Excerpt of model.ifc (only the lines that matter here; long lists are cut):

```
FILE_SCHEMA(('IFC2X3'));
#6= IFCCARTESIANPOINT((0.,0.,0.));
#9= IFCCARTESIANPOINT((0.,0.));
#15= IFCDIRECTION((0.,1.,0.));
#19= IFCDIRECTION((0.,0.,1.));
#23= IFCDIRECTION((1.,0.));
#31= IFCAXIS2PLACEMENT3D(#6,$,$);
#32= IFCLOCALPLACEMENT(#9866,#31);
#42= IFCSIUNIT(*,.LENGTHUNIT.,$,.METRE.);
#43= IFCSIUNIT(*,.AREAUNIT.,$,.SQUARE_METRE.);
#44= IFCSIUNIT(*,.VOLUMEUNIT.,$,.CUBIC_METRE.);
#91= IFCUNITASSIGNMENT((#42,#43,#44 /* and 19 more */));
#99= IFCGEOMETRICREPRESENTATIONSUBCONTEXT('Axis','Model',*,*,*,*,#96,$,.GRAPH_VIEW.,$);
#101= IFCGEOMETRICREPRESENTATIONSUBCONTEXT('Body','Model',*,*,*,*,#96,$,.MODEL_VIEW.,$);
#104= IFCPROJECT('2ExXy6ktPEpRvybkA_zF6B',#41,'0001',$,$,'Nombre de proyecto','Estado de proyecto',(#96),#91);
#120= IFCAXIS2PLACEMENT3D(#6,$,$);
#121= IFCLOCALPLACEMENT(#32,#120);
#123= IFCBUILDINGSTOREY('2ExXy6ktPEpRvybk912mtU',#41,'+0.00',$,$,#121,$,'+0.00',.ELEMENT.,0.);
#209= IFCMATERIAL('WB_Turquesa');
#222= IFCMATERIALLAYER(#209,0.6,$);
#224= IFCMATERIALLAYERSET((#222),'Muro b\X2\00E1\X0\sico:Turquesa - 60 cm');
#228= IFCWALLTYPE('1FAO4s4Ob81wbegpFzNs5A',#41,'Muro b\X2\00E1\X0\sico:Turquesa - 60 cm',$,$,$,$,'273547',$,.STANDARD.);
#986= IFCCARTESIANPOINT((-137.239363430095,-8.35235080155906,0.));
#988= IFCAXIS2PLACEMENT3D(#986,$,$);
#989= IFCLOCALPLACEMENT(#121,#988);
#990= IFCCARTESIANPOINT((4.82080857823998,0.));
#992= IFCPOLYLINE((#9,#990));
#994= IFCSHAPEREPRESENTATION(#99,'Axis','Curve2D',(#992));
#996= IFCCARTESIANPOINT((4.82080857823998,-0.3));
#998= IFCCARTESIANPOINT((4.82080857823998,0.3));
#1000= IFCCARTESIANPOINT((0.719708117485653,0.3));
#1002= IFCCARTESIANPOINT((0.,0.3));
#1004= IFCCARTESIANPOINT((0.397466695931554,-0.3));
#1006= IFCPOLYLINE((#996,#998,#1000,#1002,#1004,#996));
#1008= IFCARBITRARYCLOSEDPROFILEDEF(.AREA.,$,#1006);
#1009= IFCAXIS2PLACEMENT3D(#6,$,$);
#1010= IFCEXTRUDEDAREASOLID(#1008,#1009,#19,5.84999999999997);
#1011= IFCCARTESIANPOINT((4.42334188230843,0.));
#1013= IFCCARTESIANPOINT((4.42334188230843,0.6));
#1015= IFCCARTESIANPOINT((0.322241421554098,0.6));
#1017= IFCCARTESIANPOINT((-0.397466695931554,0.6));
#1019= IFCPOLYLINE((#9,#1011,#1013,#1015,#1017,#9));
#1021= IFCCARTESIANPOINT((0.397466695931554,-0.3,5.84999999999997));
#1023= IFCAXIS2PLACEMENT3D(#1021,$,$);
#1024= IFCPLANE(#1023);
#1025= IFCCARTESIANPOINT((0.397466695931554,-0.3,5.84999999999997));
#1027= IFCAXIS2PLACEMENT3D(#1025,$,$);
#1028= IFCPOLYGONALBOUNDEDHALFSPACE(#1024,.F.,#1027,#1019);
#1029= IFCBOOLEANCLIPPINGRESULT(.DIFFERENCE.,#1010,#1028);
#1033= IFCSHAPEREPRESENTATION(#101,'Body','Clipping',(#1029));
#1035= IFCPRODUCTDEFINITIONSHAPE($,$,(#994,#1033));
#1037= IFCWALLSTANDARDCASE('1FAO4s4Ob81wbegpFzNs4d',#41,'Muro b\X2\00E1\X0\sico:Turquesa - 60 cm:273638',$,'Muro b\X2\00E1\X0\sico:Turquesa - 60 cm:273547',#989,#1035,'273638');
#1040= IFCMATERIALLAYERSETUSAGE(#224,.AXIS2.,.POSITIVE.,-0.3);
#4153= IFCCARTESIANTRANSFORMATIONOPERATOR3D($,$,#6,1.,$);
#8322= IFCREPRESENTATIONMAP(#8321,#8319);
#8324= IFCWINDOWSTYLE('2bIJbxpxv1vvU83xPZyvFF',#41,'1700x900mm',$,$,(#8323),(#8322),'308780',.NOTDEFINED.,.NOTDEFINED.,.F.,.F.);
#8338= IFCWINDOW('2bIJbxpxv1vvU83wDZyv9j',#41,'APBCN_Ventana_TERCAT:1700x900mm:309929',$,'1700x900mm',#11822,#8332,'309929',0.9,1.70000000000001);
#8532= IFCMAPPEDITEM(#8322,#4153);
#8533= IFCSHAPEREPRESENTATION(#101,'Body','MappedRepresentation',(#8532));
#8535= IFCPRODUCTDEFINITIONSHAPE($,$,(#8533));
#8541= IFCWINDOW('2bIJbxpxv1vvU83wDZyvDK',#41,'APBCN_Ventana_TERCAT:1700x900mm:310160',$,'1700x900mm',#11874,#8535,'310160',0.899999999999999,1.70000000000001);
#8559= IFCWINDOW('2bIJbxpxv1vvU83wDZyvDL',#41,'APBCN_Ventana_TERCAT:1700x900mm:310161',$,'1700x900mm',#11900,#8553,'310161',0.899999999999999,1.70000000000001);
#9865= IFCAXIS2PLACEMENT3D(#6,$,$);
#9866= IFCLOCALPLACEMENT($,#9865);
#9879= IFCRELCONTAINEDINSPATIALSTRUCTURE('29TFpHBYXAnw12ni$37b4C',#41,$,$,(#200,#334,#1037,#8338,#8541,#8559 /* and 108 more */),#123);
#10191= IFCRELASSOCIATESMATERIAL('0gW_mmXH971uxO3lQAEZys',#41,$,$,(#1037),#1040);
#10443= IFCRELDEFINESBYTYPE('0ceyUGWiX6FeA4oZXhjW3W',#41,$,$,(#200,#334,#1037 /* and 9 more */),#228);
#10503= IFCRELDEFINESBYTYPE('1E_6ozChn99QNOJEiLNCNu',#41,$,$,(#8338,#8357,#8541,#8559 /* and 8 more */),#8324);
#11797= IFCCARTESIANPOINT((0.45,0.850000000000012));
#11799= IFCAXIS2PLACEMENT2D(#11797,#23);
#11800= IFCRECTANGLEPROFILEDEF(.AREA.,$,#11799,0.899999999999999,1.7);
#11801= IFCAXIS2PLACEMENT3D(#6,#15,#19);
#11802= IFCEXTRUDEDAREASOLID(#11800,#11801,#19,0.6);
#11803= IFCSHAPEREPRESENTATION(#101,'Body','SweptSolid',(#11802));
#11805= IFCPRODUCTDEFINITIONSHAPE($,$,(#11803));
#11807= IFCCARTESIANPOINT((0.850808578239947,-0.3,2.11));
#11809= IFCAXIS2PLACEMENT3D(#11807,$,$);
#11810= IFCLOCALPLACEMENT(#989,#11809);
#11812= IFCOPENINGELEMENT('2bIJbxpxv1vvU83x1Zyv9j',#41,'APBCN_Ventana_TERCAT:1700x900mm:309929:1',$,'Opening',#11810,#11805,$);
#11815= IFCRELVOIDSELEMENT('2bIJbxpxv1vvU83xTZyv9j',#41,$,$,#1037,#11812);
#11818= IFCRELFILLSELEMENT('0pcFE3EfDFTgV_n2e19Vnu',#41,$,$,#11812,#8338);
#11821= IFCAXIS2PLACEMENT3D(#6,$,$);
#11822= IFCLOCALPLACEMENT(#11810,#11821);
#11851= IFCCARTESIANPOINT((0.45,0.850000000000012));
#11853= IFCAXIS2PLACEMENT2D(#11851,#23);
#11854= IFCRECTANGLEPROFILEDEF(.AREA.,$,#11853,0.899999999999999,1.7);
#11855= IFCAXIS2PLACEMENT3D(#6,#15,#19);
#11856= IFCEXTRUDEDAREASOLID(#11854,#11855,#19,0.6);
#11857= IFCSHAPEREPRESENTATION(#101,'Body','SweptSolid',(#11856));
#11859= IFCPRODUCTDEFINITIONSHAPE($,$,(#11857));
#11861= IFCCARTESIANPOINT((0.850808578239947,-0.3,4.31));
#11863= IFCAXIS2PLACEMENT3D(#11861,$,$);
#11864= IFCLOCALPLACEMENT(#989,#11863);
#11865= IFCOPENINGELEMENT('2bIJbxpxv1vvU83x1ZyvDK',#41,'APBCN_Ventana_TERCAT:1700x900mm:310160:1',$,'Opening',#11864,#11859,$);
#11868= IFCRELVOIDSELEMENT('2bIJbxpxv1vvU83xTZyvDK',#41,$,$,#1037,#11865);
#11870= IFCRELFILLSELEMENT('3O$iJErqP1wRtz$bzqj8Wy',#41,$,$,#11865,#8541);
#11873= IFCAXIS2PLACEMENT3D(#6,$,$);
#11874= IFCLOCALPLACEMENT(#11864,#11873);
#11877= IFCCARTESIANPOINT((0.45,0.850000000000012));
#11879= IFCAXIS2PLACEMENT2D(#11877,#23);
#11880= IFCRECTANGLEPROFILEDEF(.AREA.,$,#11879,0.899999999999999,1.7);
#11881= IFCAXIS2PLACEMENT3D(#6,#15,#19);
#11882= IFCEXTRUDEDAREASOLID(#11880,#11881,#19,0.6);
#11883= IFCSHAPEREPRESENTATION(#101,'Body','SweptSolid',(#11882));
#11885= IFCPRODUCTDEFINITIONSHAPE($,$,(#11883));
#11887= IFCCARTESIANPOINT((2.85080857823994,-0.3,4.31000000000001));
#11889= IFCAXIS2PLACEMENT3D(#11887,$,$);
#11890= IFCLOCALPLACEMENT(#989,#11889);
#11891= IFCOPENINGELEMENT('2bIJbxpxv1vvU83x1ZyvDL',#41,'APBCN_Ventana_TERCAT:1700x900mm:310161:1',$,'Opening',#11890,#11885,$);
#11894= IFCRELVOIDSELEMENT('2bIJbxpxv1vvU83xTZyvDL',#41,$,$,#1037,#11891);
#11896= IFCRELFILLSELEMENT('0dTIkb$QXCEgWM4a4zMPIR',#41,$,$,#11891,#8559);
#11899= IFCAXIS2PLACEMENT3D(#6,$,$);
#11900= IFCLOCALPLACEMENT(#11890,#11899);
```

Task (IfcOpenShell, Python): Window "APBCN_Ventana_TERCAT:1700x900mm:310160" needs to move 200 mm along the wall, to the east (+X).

```python
import ifcopenshell
import ifcopenshell.api.geometry
import ifcopenshell.util.placement
import ifcopenshell.util.unit

model = ifcopenshell.open("model.ifc")
unit_scale = ifcopenshell.util.unit.calculate_unit_scale(model)

window = model.by_id(8541)
opening = window.FillsVoids[0].RelatingOpeningElement
wall = opening.VoidsElements[0].RelatingBuildingElement

wall_matrix = ifcopenshell.util.placement.get_local_placement(wall.ObjectPlacement)
shift = wall_matrix[:3, 0] * 0.2 / unit_scale
before = ifcopenshell.util.placement.get_local_placement(window.ObjectPlacement)[:3, 3].copy()

# The window is placed relative to its opening, so it follows when the opening moves.
matrix = ifcopenshell.util.placement.get_local_placement(opening.ObjectPlacement)
matrix[:3, 3] += shift
ifcopenshell.api.geometry.edit_object_placement(
    model, product=opening, matrix=matrix, is_si=False, should_transform_children=True
)

after = ifcopenshell.util.placement.get_local_placement(window.ObjectPlacement)[:3, 3]
print("window moved by", (after - before).round(3) + 0.0)

model.write("model_updated.ifc")
```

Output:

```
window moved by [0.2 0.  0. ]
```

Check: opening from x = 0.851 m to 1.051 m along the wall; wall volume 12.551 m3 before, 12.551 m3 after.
